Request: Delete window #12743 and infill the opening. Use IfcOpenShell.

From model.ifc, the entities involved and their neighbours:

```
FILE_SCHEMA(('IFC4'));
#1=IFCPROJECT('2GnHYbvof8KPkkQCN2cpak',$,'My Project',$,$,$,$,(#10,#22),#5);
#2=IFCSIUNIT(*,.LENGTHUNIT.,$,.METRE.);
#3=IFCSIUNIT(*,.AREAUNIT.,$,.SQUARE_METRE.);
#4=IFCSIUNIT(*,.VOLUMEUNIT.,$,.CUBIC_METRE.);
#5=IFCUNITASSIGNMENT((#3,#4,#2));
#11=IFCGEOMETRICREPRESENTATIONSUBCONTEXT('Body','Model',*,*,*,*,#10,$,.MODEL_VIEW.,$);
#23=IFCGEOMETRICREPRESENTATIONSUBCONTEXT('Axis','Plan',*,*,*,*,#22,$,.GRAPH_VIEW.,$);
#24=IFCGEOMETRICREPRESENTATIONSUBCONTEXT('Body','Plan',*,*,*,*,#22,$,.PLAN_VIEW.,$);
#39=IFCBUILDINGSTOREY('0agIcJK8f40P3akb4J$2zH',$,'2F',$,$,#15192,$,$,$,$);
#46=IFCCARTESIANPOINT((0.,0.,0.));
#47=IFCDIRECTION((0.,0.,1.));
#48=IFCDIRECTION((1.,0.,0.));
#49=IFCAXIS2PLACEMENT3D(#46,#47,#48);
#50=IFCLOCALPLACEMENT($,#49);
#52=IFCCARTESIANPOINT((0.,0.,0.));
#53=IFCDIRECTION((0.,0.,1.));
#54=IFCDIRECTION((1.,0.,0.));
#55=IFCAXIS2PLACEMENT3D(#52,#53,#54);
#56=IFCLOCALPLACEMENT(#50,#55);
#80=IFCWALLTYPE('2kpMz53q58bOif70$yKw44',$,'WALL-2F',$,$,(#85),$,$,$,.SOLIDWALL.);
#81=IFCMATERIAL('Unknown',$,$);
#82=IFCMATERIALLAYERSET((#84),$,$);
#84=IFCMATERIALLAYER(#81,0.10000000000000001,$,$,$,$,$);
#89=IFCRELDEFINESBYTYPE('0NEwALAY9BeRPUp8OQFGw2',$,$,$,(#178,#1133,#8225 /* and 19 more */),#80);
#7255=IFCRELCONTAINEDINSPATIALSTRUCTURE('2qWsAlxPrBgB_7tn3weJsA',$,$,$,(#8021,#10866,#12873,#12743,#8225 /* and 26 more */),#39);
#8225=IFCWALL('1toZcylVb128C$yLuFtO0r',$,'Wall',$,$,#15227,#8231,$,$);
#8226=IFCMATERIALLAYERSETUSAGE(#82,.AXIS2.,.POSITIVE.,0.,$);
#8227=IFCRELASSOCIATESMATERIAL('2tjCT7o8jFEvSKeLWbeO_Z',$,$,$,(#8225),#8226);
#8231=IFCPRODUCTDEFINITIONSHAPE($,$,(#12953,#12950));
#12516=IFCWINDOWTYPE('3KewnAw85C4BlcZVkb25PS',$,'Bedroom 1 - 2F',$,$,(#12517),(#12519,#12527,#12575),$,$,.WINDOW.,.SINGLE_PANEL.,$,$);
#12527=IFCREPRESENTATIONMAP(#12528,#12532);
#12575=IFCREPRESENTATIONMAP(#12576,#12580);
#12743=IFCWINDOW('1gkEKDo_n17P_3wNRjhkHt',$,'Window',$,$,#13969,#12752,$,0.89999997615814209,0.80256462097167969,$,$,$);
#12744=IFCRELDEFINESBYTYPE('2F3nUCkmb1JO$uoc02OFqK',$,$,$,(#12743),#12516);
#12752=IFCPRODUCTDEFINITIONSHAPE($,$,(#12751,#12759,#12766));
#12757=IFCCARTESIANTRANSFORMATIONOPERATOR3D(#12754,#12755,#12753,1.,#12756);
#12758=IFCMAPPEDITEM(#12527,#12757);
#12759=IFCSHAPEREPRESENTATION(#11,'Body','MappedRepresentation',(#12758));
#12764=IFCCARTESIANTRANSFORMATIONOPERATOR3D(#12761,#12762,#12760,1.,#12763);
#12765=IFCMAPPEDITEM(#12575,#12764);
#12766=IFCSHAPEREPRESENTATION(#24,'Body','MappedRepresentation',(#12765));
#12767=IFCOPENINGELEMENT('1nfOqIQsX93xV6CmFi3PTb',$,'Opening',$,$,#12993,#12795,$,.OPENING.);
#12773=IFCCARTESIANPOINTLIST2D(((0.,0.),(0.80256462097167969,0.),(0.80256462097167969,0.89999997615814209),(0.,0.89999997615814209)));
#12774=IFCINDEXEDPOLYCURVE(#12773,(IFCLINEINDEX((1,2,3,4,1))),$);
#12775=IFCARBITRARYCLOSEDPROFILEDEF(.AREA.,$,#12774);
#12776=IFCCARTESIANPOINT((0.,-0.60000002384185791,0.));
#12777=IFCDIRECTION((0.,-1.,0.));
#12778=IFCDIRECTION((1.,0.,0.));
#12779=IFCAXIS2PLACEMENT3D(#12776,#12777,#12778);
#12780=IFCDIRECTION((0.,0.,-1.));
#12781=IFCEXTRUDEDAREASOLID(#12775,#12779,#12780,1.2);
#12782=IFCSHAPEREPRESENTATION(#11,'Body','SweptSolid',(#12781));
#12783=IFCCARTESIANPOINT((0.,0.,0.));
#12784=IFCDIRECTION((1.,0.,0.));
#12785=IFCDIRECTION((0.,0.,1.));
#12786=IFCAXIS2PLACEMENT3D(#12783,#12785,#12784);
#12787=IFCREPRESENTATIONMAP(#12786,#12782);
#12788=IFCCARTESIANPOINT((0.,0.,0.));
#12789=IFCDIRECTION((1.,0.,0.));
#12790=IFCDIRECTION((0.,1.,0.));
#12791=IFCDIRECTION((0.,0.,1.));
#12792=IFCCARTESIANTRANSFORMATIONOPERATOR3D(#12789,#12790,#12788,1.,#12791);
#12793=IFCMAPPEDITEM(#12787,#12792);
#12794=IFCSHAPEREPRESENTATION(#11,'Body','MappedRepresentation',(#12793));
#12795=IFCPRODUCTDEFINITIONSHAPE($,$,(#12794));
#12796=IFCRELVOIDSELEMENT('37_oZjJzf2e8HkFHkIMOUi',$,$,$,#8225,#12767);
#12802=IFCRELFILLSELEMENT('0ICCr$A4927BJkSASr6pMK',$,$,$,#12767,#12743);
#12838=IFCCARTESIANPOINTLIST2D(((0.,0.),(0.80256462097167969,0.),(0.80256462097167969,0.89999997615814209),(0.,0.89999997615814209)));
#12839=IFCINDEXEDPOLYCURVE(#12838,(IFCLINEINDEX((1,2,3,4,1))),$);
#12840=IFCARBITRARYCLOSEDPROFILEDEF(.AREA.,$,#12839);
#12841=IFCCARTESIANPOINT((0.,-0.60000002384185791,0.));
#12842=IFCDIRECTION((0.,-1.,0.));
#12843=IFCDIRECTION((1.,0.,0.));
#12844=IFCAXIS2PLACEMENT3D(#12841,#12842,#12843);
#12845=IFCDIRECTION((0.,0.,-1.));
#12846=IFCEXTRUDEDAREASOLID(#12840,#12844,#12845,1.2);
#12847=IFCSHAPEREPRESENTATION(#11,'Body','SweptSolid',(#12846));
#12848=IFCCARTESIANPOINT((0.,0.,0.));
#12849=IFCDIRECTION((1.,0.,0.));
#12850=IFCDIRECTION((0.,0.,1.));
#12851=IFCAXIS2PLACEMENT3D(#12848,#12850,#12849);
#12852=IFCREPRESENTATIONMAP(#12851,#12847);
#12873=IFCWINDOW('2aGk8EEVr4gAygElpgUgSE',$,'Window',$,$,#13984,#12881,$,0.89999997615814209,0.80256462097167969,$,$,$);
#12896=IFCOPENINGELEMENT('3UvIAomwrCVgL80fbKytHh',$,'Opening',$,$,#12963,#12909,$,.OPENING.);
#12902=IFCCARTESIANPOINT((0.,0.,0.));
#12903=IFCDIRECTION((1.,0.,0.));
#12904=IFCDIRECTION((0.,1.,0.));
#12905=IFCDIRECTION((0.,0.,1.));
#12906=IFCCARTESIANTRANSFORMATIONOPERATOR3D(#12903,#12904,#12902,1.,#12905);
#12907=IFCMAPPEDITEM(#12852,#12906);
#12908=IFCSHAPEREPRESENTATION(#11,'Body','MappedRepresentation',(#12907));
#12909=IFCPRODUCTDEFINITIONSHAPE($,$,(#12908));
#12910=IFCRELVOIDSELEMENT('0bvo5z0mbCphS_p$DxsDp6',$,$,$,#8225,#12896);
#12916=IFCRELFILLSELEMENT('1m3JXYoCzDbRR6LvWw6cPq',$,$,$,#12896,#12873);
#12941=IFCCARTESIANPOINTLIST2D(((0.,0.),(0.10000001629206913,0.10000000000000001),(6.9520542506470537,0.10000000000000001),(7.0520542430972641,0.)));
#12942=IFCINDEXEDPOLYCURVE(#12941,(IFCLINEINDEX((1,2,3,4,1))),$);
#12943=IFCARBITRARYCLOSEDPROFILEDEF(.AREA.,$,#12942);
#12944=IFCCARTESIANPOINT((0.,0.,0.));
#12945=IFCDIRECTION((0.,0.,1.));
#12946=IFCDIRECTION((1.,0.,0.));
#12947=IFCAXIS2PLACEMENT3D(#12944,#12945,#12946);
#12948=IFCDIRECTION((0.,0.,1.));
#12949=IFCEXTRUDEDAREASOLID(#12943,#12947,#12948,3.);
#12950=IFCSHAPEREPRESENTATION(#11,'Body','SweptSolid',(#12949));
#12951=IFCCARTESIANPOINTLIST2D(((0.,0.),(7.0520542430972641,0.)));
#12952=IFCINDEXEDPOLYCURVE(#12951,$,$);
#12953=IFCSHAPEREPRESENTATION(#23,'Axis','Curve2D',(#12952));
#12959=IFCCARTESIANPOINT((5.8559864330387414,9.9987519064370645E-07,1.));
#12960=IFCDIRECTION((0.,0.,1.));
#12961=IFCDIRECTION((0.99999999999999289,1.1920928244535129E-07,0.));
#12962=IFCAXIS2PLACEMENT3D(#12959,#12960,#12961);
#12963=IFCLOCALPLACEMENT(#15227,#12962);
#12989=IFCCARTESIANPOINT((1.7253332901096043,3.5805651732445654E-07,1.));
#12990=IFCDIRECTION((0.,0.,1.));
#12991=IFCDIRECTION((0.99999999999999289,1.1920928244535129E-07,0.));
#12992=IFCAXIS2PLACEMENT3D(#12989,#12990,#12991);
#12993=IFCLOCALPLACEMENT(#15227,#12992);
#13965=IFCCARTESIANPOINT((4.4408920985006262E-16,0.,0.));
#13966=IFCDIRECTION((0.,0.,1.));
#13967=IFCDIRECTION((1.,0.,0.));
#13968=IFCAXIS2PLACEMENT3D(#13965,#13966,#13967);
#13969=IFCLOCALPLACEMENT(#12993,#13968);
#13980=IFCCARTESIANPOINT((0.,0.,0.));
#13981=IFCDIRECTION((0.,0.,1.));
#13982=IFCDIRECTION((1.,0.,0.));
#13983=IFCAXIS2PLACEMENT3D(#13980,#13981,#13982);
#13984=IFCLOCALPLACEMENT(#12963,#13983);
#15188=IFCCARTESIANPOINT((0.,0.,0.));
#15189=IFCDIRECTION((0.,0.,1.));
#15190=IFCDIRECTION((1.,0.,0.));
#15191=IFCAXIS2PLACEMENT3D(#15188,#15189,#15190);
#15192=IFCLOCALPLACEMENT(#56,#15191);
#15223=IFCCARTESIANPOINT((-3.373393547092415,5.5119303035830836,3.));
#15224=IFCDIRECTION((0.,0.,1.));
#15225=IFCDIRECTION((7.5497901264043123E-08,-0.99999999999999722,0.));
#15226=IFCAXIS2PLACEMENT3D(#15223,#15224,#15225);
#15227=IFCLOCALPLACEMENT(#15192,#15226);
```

```python
import ifcopenshell
import ifcopenshell.api.feature
import ifcopenshell.api.root
import ifcopenshell.geom
import ifcopenshell.util.shape

model = ifcopenshell.open("model.ifc")
settings = ifcopenshell.geom.settings()


def volume(element):
    """Net volume in cubic metres, openings subtracted."""
    shape = ifcopenshell.geom.create_shape(settings, element)
    return ifcopenshell.util.shape.get_volume(shape.geometry)


window = model.by_guid("1gkEKDo_n17P_3wNRjhkHt")
opening = window.FillsVoids[0].RelatingOpeningElement
wall = opening.VoidsElements[0].RelatingBuildingElement
before = volume(wall)

ifcopenshell.api.root.remove_product(model, product=window)
ifcopenshell.api.feature.remove_feature(model, feature=opening)

after = volume(wall)

print(f"wall volume {before:.3f} -> {after:.3f} m3")

model.write("model_edited.ifc")
```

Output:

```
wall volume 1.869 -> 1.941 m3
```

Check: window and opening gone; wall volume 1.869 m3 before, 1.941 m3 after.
